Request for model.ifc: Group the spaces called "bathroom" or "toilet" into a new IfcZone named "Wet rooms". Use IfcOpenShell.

First a look at what the model holds.

```python
import ifcopenshell

model = ifcopenshell.open("model.ifc")
print(model.schema)
seen = {}
for space in model.by_type("IfcSpace"):
    seen[space.LongName] = seen.get(space.LongName, 0) + 1
for name, count in sorted(seen.items(), key=str):
    print(count, "x", name)
print("zones:", [z.Name for z in model.by_type("IfcZone")][:20])
```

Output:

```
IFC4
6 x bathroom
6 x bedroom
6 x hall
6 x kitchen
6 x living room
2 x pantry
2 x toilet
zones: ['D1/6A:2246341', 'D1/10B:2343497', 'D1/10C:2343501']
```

```python
import ifcopenshell
import ifcopenshell.api.group
import ifcopenshell.api.root

model = ifcopenshell.open("model.ifc")

names = {"bathroom", "toilet"}
spaces = [s for s in model.by_type("IfcSpace") if s.LongName in names]

zone = ifcopenshell.api.root.create_entity(model, ifc_class="IfcZone", name="Wet rooms")
ifcopenshell.api.group.assign_group(model, products=spaces, group=zone)
print(len(spaces), "spaces in", zone.Name)

model.write("model_updated.ifc")
```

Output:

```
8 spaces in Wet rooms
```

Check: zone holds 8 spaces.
